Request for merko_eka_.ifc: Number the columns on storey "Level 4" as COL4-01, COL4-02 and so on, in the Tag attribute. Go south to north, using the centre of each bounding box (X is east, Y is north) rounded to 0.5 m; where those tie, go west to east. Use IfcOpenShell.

First a look at what the model holds.

```python
import ifcopenshell
import ifcopenshell.util.element
import ifcopenshell.util.placement

model = ifcopenshell.open("merko_eka_.ifc")
print(model.schema)
storey = next(s for s in model.by_type("IfcBuildingStorey") if s.Name == "Level 4")
columns = [e for e in ifcopenshell.util.element.get_decomposition(storey) if e.is_a("IfcColumn")]
for e in sorted(columns, key=lambda e: e.id()):
    origin = ifcopenshell.util.placement.get_local_placement(e.ObjectPlacement)[:3, 3]
    print(e.id(), e.Tag, e.Name, origin.round(2) + 0.0, sep=" | ")
```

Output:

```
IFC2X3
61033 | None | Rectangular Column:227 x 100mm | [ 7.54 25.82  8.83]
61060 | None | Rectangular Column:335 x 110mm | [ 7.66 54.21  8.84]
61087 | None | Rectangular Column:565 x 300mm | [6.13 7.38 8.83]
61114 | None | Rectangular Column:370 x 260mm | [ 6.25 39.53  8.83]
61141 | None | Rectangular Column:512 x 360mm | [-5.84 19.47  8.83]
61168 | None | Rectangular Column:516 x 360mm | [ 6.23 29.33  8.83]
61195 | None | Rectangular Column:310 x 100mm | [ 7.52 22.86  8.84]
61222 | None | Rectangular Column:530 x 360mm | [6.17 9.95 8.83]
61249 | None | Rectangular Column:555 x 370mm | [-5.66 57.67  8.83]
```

```python
import ifcopenshell
import ifcopenshell.geom
import ifcopenshell.util.element
import ifcopenshell.util.shape

model = ifcopenshell.open("merko_eka_.ifc")
settings = ifcopenshell.geom.settings()
settings.set("use-world-coords", True)


def centre(element):
    shape = ifcopenshell.geom.create_shape(settings, element)
    return ifcopenshell.util.shape.get_bbox_centroid(shape.geometry)


storey = next(s for s in model.by_type("IfcBuildingStorey") if s.Name == "Level 4")
columns = [e for e in ifcopenshell.util.element.get_decomposition(storey) if e.is_a("IfcColumn")]

# Insertion points can sit at a corner or the storey origin, so sort by the geometry (in metres).
centres = {e: centre(e) for e in columns}
columns.sort(key=lambda e: (round(centres[e][1] / 0.5), centres[e][0]))

for i, e in enumerate(columns, start=1):
    number = f"COL4-{i:02d}"
    e.Tag = number
    print(e.id(), number)

model.write("merko_eka_-out.ifc")
```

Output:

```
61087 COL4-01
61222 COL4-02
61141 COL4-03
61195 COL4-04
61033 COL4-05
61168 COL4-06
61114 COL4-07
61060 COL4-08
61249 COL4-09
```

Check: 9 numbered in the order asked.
